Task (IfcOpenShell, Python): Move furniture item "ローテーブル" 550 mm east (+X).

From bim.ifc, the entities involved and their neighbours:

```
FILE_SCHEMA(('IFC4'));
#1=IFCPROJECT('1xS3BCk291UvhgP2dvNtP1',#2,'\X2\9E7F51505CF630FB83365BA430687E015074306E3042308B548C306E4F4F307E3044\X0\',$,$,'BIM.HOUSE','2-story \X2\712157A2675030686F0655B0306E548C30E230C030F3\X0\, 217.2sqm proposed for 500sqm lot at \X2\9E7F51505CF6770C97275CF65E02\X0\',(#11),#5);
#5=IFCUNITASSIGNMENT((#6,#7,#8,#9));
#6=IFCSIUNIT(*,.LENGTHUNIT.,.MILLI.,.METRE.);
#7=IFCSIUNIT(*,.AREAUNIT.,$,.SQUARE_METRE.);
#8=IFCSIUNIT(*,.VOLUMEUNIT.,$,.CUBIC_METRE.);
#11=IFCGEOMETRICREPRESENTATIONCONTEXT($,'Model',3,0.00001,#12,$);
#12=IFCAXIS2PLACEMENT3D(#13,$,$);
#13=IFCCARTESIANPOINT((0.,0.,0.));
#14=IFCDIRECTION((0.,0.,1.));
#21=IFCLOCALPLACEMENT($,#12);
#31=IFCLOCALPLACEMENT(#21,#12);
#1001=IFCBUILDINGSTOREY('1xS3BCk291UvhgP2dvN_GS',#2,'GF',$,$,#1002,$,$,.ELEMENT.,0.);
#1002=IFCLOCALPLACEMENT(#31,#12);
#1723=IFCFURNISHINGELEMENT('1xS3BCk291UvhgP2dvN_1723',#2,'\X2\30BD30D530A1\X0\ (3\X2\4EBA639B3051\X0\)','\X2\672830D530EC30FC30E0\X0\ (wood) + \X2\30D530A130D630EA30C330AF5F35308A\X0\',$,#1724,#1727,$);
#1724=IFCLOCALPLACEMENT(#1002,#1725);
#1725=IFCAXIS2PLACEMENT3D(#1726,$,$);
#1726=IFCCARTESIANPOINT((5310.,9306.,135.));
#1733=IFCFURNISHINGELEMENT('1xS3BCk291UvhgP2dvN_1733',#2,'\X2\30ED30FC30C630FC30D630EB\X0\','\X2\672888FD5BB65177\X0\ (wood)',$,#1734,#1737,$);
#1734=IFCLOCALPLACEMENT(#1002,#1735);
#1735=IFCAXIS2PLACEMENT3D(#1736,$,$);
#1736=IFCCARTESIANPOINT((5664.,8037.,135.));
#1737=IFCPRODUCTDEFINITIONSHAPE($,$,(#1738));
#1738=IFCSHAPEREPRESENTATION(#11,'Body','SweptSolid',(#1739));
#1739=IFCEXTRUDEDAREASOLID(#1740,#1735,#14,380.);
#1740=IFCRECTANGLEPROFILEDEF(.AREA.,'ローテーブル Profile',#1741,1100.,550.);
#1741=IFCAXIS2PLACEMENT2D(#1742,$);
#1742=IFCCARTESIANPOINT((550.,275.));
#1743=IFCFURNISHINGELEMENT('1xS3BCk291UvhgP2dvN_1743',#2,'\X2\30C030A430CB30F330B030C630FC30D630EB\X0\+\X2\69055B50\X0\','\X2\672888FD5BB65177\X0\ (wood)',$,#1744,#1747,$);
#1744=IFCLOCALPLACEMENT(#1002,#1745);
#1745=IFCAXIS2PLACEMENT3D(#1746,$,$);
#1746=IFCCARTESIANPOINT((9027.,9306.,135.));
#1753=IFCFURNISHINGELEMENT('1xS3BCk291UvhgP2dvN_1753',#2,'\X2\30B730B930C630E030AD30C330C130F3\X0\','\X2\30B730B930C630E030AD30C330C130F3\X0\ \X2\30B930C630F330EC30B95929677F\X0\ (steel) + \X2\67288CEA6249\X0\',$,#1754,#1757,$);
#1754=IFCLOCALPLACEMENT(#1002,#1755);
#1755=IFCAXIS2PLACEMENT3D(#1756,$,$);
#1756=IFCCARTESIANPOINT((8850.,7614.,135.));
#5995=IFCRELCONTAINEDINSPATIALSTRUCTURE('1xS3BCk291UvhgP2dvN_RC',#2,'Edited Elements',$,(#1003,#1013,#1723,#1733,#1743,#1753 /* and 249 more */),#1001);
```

```python
import ifcopenshell
import ifcopenshell.api.geometry
import ifcopenshell.util.placement

model = ifcopenshell.open("bim.ifc")

item = model.by_guid("1xS3BCk291UvhgP2dvN_1733")
matrix = ifcopenshell.util.placement.get_local_placement(item.ObjectPlacement)
matrix[0, 3] += 550.0
ifcopenshell.api.geometry.edit_object_placement(model, product=item, matrix=matrix, is_si=False)

print(ifcopenshell.util.placement.get_local_placement(item.ObjectPlacement).round(3) + 0.0)

model.write("bim_updated.ifc")
```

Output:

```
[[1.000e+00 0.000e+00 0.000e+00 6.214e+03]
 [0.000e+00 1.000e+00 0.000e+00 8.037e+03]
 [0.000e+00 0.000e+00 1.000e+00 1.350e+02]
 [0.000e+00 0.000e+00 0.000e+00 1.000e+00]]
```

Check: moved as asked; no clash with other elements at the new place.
